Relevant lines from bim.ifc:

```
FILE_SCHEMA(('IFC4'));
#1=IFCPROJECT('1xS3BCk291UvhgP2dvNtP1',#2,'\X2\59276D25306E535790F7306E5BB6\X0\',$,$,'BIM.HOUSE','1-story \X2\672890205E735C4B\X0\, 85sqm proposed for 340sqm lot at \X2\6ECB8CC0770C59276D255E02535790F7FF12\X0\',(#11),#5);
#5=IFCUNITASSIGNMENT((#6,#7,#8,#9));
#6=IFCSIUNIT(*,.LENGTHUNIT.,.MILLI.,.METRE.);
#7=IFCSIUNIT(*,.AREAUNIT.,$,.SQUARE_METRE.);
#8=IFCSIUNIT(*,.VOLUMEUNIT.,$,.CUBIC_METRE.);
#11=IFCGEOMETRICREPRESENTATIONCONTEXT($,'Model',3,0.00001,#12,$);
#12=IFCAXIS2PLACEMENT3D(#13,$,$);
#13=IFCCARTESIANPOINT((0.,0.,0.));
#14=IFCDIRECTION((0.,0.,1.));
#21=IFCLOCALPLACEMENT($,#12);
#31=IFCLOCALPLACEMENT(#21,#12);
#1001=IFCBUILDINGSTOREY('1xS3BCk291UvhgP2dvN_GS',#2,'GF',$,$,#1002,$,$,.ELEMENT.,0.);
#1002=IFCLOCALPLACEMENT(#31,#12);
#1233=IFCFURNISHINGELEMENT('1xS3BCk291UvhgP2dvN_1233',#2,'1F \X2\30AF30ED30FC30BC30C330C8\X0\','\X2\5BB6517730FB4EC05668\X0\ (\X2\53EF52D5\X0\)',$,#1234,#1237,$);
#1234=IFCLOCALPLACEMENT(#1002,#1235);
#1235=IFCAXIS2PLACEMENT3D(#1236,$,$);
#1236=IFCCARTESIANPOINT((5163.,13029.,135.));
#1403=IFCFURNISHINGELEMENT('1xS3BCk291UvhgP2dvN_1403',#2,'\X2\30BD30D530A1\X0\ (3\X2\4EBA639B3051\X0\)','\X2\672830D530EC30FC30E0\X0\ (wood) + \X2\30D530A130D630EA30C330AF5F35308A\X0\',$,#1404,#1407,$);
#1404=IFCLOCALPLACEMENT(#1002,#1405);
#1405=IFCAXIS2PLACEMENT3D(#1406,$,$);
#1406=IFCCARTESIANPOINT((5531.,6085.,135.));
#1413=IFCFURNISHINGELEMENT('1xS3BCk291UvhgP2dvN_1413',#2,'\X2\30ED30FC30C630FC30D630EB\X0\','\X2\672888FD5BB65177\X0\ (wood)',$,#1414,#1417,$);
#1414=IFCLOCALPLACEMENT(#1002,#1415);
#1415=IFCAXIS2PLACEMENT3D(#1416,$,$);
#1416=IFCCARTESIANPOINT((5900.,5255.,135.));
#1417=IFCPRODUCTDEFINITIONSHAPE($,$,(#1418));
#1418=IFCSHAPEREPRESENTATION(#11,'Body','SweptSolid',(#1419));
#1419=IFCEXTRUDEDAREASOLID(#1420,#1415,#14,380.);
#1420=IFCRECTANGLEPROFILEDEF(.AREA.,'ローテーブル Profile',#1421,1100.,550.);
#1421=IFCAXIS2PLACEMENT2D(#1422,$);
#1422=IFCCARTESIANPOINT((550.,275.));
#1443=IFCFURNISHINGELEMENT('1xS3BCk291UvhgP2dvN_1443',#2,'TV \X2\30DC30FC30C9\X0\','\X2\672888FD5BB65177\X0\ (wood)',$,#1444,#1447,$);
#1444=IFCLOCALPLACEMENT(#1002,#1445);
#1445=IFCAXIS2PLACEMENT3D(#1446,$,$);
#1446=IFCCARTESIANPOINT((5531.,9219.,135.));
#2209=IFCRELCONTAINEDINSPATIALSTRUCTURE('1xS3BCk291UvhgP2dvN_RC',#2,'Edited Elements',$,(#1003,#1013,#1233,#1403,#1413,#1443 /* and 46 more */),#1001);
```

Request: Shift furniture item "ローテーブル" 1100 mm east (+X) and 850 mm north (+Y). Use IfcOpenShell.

```python
import ifcopenshell
import ifcopenshell.api.geometry
import ifcopenshell.util.placement

model = ifcopenshell.open("bim.ifc")

item = model.by_id(1413)
matrix = ifcopenshell.util.placement.get_local_placement(item.ObjectPlacement)
matrix[0, 3] += 1100.0
matrix[1, 3] += 850.0
ifcopenshell.api.geometry.edit_object_placement(model, product=item, matrix=matrix, is_si=False)

print(ifcopenshell.util.placement.get_local_placement(item.ObjectPlacement).round(3) + 0.0)

model.write("bim_rev.ifc")
```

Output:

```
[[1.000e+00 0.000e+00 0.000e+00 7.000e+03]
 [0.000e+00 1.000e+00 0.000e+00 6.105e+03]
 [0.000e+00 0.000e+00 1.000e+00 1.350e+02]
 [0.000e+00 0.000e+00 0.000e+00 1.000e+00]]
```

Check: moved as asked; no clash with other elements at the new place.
